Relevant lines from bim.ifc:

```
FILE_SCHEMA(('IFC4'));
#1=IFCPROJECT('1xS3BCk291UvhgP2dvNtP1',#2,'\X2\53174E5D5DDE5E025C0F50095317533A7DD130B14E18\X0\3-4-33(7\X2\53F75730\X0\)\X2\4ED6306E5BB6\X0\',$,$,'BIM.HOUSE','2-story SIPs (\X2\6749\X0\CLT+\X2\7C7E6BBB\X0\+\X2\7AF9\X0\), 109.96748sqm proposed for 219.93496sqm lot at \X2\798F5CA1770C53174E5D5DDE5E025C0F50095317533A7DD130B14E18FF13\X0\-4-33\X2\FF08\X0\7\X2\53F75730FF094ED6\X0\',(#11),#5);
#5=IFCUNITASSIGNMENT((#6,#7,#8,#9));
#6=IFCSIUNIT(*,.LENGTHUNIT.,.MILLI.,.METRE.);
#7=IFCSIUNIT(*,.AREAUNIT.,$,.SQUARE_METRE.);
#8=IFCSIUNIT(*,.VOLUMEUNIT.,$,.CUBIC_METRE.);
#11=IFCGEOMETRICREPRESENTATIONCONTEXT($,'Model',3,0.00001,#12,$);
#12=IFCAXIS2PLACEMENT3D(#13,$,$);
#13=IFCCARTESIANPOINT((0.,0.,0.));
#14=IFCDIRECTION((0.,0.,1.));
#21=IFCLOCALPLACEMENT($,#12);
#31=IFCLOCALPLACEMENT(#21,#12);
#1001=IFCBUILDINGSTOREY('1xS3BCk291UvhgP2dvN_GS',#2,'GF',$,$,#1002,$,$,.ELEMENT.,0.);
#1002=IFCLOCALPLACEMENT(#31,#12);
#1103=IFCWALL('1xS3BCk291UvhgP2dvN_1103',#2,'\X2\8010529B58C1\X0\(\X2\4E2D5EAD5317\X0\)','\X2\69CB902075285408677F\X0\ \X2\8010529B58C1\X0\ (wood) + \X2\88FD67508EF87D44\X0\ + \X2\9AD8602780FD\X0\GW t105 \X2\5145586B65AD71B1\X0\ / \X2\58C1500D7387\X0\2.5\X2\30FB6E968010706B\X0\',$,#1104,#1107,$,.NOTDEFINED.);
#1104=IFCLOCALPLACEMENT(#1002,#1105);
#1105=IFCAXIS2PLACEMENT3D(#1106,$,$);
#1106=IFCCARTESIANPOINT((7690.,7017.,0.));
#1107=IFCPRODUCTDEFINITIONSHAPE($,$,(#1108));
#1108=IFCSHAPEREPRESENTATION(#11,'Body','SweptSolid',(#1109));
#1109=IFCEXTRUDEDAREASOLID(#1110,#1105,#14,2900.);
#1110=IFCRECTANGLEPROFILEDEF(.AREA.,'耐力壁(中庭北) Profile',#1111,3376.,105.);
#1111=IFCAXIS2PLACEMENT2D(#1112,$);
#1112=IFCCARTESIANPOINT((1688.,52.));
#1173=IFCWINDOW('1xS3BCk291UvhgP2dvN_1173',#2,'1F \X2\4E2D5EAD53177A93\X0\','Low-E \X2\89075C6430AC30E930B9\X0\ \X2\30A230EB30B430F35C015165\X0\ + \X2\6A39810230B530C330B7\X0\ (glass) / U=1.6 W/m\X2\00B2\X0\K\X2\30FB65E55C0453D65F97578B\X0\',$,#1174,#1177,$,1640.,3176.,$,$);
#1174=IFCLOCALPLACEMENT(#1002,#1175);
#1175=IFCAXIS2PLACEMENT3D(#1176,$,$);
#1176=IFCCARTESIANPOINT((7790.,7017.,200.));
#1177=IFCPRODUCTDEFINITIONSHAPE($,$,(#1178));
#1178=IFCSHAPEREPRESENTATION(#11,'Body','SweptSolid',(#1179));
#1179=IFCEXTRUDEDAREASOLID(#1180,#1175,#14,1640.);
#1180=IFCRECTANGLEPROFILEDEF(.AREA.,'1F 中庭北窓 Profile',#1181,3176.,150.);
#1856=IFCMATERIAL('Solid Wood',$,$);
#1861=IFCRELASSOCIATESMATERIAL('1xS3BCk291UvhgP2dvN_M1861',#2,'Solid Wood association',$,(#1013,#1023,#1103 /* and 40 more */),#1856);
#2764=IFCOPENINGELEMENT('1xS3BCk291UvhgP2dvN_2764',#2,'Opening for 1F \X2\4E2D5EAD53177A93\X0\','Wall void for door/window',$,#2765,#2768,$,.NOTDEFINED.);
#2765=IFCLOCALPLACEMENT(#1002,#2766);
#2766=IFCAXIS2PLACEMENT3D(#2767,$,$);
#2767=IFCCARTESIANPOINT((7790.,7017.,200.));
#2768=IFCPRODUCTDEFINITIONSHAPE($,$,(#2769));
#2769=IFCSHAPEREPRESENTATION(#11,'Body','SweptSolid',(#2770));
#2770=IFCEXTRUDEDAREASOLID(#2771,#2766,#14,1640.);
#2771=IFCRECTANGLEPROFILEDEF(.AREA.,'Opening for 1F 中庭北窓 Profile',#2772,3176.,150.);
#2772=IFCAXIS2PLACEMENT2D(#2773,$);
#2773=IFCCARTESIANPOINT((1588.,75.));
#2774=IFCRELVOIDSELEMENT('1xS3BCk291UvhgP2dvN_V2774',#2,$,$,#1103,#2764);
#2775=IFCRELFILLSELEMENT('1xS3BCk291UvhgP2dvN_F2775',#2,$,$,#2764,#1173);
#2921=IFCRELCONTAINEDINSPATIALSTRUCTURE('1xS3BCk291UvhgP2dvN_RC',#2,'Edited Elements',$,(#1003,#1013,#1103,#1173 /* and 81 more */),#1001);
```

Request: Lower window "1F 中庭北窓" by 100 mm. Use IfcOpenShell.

```python
import numpy as np
import ifcopenshell
import ifcopenshell.api.geometry
import ifcopenshell.util.placement
import ifcopenshell.util.unit

model = ifcopenshell.open("bim.ifc")
unit_scale = ifcopenshell.util.unit.calculate_unit_scale(model)

window = model.by_guid("1xS3BCk291UvhgP2dvN_1173")
opening = window.FillsVoids[0].RelatingOpeningElement
dz = -0.1 / unit_scale

shift = np.array([0.0, 0.0, dz])
# The window is not placed relative to its opening, so move both.
for product in (opening, window):
    matrix = ifcopenshell.util.placement.get_local_placement(product.ObjectPlacement)
    matrix[:3, 3] += shift
    ifcopenshell.api.geometry.edit_object_placement(model, product=product, matrix=matrix, is_si=False)

print(f"moved by {dz * unit_scale:+.3f} m")

model.write("bim_v2.ifc")
```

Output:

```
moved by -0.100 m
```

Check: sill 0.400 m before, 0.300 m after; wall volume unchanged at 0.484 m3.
